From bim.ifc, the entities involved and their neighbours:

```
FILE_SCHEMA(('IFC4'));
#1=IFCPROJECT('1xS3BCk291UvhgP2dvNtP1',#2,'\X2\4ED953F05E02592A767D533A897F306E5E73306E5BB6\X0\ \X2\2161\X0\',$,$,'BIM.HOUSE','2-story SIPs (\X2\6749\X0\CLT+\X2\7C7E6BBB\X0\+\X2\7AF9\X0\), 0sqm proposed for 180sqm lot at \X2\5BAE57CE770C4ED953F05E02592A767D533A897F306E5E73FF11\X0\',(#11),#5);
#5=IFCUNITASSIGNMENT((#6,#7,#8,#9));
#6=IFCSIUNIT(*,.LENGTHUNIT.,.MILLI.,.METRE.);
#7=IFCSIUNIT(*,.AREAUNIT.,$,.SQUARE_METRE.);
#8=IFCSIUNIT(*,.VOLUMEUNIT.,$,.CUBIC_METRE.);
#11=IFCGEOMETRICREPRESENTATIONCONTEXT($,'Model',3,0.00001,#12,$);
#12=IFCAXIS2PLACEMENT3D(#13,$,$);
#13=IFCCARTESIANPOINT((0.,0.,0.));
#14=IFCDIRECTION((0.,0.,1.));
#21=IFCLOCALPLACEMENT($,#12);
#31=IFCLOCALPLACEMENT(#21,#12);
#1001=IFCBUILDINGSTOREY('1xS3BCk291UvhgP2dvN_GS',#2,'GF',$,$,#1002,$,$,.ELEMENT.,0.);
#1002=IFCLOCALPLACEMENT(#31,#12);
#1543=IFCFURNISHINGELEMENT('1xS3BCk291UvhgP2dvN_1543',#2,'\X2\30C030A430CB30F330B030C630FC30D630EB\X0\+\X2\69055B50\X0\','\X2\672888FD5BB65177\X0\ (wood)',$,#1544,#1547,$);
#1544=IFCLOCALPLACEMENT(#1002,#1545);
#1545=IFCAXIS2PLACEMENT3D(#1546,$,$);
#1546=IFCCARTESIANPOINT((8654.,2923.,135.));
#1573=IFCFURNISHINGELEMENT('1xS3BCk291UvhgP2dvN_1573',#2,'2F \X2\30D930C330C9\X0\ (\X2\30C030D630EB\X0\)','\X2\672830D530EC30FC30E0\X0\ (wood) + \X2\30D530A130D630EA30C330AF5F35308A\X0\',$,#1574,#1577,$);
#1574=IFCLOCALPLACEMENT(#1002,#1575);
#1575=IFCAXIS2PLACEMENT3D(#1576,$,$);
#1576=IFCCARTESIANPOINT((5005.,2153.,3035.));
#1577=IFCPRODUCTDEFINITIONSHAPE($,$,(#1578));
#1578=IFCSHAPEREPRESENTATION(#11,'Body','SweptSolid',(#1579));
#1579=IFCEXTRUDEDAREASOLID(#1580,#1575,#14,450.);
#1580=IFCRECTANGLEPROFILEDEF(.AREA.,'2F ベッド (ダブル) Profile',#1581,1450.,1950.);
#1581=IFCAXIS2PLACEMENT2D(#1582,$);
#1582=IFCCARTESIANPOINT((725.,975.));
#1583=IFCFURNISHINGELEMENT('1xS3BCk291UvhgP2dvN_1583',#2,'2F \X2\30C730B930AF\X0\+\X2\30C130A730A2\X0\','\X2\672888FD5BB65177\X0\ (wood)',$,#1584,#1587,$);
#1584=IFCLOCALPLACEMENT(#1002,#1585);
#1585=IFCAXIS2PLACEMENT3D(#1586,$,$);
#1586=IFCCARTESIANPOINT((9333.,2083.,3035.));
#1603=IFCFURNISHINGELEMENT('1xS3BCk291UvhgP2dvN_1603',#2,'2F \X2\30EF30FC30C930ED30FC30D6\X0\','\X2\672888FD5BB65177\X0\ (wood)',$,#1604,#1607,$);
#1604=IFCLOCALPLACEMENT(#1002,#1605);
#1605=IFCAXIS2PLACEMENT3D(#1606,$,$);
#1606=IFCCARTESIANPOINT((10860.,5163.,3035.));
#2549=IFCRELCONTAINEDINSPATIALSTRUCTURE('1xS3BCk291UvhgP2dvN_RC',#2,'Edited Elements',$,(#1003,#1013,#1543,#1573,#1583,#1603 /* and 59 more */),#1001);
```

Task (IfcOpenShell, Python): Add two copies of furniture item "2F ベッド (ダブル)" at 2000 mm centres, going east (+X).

```python
import numpy as np
import ifcopenshell
import ifcopenshell.api.geometry
import ifcopenshell.api.root
import ifcopenshell.util.element
import ifcopenshell.util.placement
import ifcopenshell.util.unit

model = ifcopenshell.open("bim.ifc")
unit_scale = ifcopenshell.util.unit.calculate_unit_scale(model)


def reuse_history(source, copy):
    """copy_class also copies each property set's owner history, people and application; keep the originals."""
    for rel in copy.IsDefinedBy:
        if rel.is_a("IfcRelDefinesByProperties") and (history := rel.RelatingPropertyDefinition.OwnerHistory):
            rel.RelatingPropertyDefinition.OwnerHistory = source.OwnerHistory
            ifcopenshell.util.element.remove_deep2(model, history)


source = model.by_id(1573)
base = ifcopenshell.util.placement.get_local_placement(source.ObjectPlacement)
step = np.array([1.0, 0.0, 0.0]) * 2 / unit_scale

for i in range(1, 3):
    copy = ifcopenshell.api.root.copy_class(model, product=source)
    copy.Representation = ifcopenshell.util.element.copy_deep(
        model, source.Representation, exclude=["IfcGeometricRepresentationContext", "IfcRepresentationMap"]
    )
    reuse_history(source, copy)
    matrix = base.copy()
    matrix[:3, 3] += i * step
    print("added at", matrix[:3, 3].round(3) + 0.0)
    ifcopenshell.api.geometry.edit_object_placement(model, product=copy, matrix=matrix, is_si=False)

model.write("bim_updated.ifc")
```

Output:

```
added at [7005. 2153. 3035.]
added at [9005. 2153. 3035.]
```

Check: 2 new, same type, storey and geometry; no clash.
